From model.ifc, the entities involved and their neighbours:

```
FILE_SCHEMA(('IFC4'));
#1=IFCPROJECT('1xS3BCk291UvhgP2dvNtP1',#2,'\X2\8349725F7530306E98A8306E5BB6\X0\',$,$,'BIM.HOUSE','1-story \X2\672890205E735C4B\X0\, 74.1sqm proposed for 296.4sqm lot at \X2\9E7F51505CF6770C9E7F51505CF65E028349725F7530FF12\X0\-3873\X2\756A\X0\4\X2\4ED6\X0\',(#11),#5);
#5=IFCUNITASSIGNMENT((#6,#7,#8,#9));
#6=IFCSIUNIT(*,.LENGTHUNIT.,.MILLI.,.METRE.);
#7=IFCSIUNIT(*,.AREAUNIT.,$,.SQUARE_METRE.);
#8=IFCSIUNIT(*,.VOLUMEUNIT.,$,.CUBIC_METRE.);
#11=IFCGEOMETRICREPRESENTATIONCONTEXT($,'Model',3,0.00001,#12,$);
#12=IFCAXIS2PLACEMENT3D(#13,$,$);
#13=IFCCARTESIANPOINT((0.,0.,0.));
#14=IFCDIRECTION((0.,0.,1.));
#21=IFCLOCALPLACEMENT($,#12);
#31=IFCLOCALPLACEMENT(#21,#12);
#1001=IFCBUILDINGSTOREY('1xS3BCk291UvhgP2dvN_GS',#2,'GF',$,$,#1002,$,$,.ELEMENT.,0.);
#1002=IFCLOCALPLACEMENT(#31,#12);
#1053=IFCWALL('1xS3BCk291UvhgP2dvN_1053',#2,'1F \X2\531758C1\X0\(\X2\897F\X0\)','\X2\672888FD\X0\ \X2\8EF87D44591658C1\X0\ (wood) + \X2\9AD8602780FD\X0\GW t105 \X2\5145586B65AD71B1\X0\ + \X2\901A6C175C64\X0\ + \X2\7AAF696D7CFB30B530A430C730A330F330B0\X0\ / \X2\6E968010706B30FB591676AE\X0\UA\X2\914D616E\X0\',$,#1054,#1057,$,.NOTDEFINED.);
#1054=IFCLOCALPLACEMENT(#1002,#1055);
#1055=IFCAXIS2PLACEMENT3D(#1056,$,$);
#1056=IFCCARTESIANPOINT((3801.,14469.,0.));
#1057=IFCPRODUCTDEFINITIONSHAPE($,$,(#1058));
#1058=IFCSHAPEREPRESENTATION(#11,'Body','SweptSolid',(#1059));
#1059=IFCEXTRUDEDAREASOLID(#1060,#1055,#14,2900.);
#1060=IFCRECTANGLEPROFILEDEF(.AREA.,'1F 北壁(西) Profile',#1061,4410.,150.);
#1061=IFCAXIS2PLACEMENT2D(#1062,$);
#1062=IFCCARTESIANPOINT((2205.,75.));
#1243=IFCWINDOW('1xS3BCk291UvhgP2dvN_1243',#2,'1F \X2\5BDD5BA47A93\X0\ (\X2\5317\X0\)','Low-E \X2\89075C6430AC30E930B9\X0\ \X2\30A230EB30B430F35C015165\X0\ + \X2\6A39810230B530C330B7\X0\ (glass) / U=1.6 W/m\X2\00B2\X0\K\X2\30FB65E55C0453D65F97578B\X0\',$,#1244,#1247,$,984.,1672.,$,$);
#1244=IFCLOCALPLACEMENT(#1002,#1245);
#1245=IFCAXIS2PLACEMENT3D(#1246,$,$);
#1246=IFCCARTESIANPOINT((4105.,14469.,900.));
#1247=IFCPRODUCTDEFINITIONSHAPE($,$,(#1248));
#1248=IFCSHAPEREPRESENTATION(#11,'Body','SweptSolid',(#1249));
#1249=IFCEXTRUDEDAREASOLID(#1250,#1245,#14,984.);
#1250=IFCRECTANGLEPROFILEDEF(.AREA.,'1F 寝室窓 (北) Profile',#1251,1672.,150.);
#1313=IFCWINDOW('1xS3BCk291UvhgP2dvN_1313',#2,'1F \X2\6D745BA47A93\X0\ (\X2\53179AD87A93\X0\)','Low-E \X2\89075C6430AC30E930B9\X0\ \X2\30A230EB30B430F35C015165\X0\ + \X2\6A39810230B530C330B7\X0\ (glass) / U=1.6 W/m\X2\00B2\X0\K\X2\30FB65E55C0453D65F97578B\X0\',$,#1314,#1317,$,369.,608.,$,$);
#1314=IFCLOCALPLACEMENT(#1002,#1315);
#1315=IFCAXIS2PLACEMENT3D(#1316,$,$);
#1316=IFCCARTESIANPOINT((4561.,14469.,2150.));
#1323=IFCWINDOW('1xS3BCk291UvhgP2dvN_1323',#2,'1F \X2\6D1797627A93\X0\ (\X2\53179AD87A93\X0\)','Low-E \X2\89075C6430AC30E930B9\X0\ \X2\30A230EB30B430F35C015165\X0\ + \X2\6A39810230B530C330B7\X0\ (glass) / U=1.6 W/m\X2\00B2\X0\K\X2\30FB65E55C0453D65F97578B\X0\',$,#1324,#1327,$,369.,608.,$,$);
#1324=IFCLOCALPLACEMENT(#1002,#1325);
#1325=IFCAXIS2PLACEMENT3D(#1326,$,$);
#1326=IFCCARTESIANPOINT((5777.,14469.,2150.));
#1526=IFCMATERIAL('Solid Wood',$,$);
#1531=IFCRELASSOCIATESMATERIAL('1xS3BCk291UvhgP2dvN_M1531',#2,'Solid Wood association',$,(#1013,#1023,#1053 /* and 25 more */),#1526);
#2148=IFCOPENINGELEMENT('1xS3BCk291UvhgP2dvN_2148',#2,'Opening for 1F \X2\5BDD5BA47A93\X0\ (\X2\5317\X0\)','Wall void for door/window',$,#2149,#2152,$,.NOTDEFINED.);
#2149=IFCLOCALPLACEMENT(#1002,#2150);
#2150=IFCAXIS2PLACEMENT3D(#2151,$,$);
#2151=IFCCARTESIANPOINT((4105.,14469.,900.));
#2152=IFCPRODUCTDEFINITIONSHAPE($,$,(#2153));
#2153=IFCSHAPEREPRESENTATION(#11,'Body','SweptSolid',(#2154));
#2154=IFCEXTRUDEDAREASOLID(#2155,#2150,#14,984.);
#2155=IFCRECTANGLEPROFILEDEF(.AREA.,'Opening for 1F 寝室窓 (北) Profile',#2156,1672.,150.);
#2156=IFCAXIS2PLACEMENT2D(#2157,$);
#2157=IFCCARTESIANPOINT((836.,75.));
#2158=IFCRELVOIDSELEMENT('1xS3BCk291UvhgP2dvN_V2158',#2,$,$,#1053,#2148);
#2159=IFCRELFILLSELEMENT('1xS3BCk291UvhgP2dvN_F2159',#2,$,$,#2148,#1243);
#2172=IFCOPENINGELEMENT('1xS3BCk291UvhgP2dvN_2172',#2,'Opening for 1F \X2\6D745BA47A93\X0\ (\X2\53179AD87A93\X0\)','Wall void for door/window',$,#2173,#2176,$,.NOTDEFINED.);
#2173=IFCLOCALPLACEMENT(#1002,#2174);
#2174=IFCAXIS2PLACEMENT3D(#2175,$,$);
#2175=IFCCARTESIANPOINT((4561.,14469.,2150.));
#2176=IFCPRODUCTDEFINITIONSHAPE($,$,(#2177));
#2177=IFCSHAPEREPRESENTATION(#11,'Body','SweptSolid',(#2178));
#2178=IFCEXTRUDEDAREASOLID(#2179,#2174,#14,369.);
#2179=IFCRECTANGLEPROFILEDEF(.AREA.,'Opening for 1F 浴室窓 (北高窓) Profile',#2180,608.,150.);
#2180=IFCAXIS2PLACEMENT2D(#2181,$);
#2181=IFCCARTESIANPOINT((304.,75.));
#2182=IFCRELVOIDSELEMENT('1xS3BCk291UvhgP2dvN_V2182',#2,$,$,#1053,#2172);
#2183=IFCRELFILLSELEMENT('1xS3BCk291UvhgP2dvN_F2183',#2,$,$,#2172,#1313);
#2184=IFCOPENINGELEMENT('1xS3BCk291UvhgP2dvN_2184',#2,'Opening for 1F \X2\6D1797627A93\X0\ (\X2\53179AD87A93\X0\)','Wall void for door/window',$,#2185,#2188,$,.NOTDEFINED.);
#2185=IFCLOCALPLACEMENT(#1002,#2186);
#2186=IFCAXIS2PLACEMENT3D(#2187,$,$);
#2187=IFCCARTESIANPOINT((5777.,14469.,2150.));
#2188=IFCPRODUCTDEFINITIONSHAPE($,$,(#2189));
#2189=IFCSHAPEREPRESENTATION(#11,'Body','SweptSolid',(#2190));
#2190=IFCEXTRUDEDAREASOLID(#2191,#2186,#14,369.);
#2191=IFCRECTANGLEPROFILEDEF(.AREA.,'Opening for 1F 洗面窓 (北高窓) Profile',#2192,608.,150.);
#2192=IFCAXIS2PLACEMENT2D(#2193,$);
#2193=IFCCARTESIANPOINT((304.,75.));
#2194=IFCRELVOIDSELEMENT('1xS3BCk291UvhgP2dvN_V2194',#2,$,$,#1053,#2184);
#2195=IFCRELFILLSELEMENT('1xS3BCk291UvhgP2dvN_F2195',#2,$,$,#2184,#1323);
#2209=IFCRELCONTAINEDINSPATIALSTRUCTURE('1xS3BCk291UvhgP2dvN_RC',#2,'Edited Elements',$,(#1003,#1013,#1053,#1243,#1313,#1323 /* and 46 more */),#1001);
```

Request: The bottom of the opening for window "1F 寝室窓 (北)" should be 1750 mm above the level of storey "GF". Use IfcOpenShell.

```python
import numpy as np
import ifcopenshell
import ifcopenshell.api.geometry
import ifcopenshell.geom
import ifcopenshell.util.element
import ifcopenshell.util.placement
import ifcopenshell.util.shape
import ifcopenshell.util.unit

model = ifcopenshell.open("model.ifc")
unit_scale = ifcopenshell.util.unit.calculate_unit_scale(model)

window = model.by_guid("1xS3BCk291UvhgP2dvN_1243")
opening = window.FillsVoids[0].RelatingOpeningElement
storey = ifcopenshell.util.element.get_container(window, ifc_class="IfcBuildingStorey")
level = ifcopenshell.util.placement.get_local_placement(storey.ObjectPlacement)[2, 3]

# The opening's origin need not be at the sill, so measure its lowest point.
shape = ifcopenshell.geom.create_shape(ifcopenshell.geom.settings(), opening)
bottom = ifcopenshell.util.shape.get_shape_bottom_elevation(shape, shape.geometry) / unit_scale
dz = level + 1.75 / unit_scale - bottom

shift = np.array([0.0, 0.0, dz])
# The window is not placed relative to its opening, so move both.
for product in (opening, window):
    matrix = ifcopenshell.util.placement.get_local_placement(product.ObjectPlacement)
    matrix[:3, 3] += shift
    ifcopenshell.api.geometry.edit_object_placement(model, product=product, matrix=matrix, is_si=False)

print(f"moved by {dz * unit_scale:+.3f} m")

model.write("model_updated.ifc")
```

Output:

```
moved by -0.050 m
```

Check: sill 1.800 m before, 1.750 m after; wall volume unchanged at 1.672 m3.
